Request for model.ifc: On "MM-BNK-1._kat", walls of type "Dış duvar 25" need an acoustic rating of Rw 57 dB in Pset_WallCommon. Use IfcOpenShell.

First a look at what the model holds.

```python
import ifcopenshell
import ifcopenshell.util.element

model = ifcopenshell.open("model.ifc")
print(model.schema)
storey = next(s for s in model.by_type("IfcBuildingStorey") if s.Name == "MM-BNK-1._kat")
walls = [e for e in ifcopenshell.util.element.get_decomposition(storey) if e.is_a("IfcWall")]
seen = {}
for e in walls:
    element_type = ifcopenshell.util.element.get_type(e)
    key = (element_type.Name if element_type != e and element_type else None, ifcopenshell.util.element.get_pset(e, "Pset_WallCommon", "AcousticRating"))
    seen[key] = seen.get(key, 0) + 1
for (name, value), count in sorted(seen.items(), key=str):
    print(count, "x", name, "|", value)
```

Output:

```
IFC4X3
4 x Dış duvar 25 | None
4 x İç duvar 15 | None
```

```python
import ifcopenshell
import ifcopenshell.api.pset
import ifcopenshell.util.element

model = ifcopenshell.open("model.ifc")

storey = next(s for s in model.by_type("IfcBuildingStorey") if s.Name == "MM-BNK-1._kat")
walls = [e for e in ifcopenshell.util.element.get_decomposition(storey) if e.is_a("IfcWall")]

count = 0
for e in walls:
    element_type = ifcopenshell.util.element.get_type(e)
    if element_type in (None, e) or element_type.Name != "Dış duvar 25":
        continue
    # add_pset returns the element's existing set when there is one.
    pset = ifcopenshell.api.pset.add_pset(model, product=e, name="Pset_WallCommon")
    ifcopenshell.api.pset.edit_pset(model, pset=pset, properties={"AcousticRating": "Rw 57 dB"})
    count += 1

print(count, "walls updated")

model.write("model_v2.ifc")
```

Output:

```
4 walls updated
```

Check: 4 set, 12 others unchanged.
